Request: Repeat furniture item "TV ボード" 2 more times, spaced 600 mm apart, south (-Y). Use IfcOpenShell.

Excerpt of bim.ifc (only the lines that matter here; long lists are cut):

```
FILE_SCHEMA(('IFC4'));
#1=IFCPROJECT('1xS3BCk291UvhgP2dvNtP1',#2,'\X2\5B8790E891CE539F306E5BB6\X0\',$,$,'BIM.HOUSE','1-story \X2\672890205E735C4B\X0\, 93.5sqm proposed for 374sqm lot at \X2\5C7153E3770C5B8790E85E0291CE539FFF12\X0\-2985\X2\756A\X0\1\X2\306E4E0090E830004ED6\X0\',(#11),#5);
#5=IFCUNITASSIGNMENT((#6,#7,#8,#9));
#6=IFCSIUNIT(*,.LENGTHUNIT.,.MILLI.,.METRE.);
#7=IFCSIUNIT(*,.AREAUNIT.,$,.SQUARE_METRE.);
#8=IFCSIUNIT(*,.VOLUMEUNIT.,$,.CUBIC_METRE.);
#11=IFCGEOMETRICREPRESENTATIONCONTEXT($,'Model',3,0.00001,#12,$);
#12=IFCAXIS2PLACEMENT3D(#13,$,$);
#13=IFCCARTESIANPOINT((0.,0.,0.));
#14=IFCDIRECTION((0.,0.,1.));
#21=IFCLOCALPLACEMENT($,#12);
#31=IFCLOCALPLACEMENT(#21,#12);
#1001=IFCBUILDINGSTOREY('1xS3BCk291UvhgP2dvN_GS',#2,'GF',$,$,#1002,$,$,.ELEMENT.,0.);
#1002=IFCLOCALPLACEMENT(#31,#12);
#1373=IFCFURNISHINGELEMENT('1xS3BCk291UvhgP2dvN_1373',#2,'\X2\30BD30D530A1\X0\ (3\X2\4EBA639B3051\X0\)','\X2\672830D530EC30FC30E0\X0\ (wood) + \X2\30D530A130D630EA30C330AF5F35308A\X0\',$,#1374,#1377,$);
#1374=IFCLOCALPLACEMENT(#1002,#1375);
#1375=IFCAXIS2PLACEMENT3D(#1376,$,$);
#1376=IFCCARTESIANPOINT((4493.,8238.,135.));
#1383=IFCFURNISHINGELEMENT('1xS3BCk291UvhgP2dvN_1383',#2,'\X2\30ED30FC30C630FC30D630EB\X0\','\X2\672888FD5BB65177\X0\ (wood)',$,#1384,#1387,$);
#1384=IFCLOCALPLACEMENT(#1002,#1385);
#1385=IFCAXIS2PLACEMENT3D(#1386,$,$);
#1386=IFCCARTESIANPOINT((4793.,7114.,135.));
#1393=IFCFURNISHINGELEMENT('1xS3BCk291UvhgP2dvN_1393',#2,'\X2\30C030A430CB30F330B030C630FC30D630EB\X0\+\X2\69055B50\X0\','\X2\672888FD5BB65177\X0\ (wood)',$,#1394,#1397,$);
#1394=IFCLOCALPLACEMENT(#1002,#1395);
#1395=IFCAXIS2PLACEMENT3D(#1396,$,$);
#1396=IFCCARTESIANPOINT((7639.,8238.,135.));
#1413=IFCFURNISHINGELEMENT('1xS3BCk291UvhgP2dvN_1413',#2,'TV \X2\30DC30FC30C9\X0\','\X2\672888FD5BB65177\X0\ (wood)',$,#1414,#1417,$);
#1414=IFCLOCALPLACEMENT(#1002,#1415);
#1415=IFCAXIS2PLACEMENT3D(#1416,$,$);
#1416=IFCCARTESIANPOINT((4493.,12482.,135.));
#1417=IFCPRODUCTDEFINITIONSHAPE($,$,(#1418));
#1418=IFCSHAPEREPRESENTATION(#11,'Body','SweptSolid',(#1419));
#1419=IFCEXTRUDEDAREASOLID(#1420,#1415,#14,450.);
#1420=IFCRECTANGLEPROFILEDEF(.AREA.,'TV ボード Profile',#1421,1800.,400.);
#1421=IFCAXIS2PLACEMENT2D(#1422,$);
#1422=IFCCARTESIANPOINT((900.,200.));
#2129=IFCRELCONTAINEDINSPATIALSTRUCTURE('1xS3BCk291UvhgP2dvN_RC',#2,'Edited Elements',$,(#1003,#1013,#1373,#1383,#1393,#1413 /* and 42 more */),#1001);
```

```python
import numpy as np
import ifcopenshell
import ifcopenshell.api.geometry
import ifcopenshell.api.root
import ifcopenshell.util.element
import ifcopenshell.util.placement
import ifcopenshell.util.unit

model = ifcopenshell.open("bim.ifc")
unit_scale = ifcopenshell.util.unit.calculate_unit_scale(model)


def reuse_history(source, copy):
    """copy_class also copies each property set's owner history, people and application; keep the originals."""
    for rel in copy.IsDefinedBy:
        if rel.is_a("IfcRelDefinesByProperties") and (history := rel.RelatingPropertyDefinition.OwnerHistory):
            rel.RelatingPropertyDefinition.OwnerHistory = source.OwnerHistory
            ifcopenshell.util.element.remove_deep2(model, history)


source = model.by_guid("1xS3BCk291UvhgP2dvN_1413")
base = ifcopenshell.util.placement.get_local_placement(source.ObjectPlacement)
step = np.array([0.0, -1.0, 0.0]) * 0.6 / unit_scale

for i in range(1, 3):
    copy = ifcopenshell.api.root.copy_class(model, product=source)
    copy.Representation = ifcopenshell.util.element.copy_deep(
        model, source.Representation, exclude=["IfcGeometricRepresentationContext", "IfcRepresentationMap"]
    )
    reuse_history(source, copy)
    matrix = base.copy()
    matrix[:3, 3] += i * step
    print("added at", matrix[:3, 3].round(3) + 0.0)
    ifcopenshell.api.geometry.edit_object_placement(model, product=copy, matrix=matrix, is_si=False)

model.write("bim_edited.ifc")
```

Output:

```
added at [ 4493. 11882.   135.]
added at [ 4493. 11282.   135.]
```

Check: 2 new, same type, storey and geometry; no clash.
